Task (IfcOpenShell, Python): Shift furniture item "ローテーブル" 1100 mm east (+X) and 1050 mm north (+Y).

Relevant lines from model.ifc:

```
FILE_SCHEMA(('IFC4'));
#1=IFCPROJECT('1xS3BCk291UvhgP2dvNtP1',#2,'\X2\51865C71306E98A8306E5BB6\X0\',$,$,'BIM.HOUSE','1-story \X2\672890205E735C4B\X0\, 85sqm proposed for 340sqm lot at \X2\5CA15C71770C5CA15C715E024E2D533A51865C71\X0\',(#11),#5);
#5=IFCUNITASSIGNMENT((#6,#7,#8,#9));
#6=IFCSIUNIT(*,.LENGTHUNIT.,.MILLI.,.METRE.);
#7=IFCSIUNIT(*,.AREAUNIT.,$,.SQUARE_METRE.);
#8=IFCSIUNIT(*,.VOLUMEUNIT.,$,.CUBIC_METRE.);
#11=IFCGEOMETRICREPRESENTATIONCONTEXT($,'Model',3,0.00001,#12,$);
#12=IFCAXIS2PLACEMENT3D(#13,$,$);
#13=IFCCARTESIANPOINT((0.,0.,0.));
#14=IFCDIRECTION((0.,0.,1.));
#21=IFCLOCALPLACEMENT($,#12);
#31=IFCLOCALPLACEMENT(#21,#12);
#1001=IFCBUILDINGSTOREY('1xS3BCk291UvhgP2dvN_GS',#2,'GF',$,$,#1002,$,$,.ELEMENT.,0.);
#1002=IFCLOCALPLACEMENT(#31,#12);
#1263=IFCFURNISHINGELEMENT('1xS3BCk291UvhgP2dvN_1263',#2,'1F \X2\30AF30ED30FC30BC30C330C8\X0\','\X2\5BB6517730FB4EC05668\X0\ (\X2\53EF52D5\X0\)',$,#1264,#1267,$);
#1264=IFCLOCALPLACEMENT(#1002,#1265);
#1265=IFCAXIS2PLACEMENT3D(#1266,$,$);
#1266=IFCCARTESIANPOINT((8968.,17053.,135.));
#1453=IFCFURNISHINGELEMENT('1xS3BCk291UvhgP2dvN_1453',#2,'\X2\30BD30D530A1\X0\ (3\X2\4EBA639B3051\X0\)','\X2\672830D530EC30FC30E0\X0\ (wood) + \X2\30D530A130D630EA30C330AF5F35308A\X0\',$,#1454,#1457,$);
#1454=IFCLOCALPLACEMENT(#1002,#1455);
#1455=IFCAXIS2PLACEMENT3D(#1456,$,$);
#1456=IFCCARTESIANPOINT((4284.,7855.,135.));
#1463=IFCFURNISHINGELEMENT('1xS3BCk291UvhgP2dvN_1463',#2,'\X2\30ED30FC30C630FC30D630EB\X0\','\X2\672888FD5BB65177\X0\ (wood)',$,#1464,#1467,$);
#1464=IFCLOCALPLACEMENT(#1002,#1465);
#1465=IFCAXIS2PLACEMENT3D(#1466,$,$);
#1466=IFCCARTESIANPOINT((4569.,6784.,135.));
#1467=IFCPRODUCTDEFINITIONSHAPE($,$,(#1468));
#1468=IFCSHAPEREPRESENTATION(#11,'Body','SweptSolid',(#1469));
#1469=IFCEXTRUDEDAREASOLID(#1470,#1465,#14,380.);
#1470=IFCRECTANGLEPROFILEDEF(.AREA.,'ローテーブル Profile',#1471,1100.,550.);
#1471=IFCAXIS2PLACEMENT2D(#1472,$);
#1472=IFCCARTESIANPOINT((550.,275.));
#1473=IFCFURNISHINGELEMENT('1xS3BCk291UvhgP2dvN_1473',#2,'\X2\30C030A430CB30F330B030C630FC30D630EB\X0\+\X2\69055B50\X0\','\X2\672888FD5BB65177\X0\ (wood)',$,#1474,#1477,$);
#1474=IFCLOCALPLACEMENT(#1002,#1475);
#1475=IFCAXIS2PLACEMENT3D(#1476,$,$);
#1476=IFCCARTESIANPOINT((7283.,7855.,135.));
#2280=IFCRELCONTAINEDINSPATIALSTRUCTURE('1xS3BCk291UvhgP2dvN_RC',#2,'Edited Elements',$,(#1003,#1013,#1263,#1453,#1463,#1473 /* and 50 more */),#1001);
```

```python
import ifcopenshell
import ifcopenshell.api.geometry
import ifcopenshell.util.placement
import ifcopenshell.util.unit

model = ifcopenshell.open("model.ifc")
unit_scale = ifcopenshell.util.unit.calculate_unit_scale(model)

item = model.by_guid("1xS3BCk291UvhgP2dvN_1463")
matrix = ifcopenshell.util.placement.get_local_placement(item.ObjectPlacement)
matrix[0, 3] += 1.1 / unit_scale
matrix[1, 3] += 1.05 / unit_scale
ifcopenshell.api.geometry.edit_object_placement(model, product=item, matrix=matrix, is_si=False)

print(ifcopenshell.util.placement.get_local_placement(item.ObjectPlacement).round(3) + 0.0)

model.write("model_edited.ifc")
```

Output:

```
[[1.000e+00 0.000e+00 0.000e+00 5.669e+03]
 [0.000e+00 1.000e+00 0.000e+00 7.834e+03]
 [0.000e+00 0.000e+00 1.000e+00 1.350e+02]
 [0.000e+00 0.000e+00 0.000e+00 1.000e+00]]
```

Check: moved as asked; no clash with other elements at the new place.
